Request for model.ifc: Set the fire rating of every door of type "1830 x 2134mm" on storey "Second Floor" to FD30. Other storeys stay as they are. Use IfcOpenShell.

First a look at what the model holds.

```python
import ifcopenshell
import ifcopenshell.util.element

model = ifcopenshell.open("model.ifc")
print(model.schema)
storey = next(s for s in model.by_type("IfcBuildingStorey") if s.Name == "Second Floor")
doors = [e for e in ifcopenshell.util.element.get_decomposition(storey) if e.is_a("IfcDoor")]
seen = {}
for e in doors:
    element_type = ifcopenshell.util.element.get_type(e)
    key = (element_type.Name if element_type != e and element_type else None, ifcopenshell.util.element.get_pset(e, "Pset_DoorCommon", "FireRating"))
    seen[key] = seen.get(key, 0) + 1
for (name, value), count in sorted(seen.items(), key=str):
    print(count, "x", name, "|", value)
```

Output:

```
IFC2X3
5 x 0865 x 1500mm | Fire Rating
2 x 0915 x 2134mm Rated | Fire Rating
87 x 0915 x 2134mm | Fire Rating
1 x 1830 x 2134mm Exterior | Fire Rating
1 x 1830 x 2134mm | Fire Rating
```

```python
import ifcopenshell
import ifcopenshell.api.pset
import ifcopenshell.util.element

model = ifcopenshell.open("model.ifc")

storey = next(s for s in model.by_type("IfcBuildingStorey") if s.Name == "Second Floor")
doors = [e for e in ifcopenshell.util.element.get_decomposition(storey) if e.is_a("IfcDoor")]

count = 0
for e in doors:
    element_type = ifcopenshell.util.element.get_type(e)
    if element_type in (None, e) or element_type.Name != "1830 x 2134mm":
        continue
    # add_pset returns the element's existing set when there is one.
    pset = ifcopenshell.api.pset.add_pset(model, product=e, name="Pset_DoorCommon")
    ifcopenshell.api.pset.edit_pset(model, pset=pset, properties={"FireRating": "FD30"})
    count += 1

print(count, "doors updated")

model.write("model_v2.ifc")
```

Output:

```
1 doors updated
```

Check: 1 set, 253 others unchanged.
